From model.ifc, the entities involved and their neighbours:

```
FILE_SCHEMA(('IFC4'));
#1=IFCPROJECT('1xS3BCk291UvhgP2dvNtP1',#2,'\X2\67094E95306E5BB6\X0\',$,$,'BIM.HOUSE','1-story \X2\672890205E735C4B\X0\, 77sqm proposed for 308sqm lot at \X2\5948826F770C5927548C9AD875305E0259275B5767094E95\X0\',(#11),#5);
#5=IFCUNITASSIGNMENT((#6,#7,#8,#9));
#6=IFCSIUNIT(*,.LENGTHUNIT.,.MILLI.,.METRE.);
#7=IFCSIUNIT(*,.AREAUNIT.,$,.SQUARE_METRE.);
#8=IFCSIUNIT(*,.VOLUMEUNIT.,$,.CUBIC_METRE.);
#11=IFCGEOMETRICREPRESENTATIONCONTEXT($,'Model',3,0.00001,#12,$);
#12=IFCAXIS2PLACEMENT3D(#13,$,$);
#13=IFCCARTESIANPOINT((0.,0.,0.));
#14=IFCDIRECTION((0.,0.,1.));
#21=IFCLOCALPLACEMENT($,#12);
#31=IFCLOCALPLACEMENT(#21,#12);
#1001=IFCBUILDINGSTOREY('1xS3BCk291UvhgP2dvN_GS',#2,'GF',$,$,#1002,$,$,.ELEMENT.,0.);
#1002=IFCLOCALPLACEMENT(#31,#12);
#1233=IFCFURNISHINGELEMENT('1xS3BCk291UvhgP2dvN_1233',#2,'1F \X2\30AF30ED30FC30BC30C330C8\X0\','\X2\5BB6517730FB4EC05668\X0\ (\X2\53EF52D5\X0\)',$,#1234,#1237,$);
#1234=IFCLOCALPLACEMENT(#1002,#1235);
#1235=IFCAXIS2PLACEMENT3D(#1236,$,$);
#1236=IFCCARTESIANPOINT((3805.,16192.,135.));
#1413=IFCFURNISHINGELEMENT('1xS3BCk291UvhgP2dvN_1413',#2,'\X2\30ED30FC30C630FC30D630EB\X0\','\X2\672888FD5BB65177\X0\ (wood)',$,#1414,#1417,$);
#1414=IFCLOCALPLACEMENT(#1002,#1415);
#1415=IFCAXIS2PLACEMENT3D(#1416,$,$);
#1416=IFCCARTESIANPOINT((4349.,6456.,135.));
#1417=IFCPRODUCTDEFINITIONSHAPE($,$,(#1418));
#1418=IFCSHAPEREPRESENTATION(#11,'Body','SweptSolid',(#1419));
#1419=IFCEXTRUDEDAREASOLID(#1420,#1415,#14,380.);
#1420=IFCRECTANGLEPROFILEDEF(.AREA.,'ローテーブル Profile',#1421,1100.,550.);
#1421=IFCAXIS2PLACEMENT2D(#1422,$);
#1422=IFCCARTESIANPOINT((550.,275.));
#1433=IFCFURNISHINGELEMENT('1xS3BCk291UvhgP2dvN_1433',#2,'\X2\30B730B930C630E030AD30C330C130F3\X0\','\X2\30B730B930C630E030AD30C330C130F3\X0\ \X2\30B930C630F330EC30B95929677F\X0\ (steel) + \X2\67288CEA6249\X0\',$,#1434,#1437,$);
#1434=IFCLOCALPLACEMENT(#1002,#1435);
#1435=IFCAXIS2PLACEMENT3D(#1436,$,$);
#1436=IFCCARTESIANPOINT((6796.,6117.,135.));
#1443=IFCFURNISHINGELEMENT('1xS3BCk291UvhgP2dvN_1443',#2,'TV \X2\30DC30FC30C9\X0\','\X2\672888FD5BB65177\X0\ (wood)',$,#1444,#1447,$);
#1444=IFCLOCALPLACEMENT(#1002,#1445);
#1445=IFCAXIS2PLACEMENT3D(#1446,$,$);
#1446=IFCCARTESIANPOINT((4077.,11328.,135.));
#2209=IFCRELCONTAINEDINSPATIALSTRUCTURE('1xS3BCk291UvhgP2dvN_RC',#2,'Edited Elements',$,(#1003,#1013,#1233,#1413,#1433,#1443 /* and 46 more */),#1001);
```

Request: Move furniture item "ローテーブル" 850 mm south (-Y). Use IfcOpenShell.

```python
import ifcopenshell
import ifcopenshell.api.geometry
import ifcopenshell.util.placement
import ifcopenshell.util.unit

model = ifcopenshell.open("model.ifc")
unit_scale = ifcopenshell.util.unit.calculate_unit_scale(model)

item = model.by_guid("1xS3BCk291UvhgP2dvN_1413")
matrix = ifcopenshell.util.placement.get_local_placement(item.ObjectPlacement)
matrix[1, 3] -= 0.85 / unit_scale
ifcopenshell.api.geometry.edit_object_placement(model, product=item, matrix=matrix, is_si=False)

print(ifcopenshell.util.placement.get_local_placement(item.ObjectPlacement).round(3) + 0.0)

model.write("model_updated.ifc")
```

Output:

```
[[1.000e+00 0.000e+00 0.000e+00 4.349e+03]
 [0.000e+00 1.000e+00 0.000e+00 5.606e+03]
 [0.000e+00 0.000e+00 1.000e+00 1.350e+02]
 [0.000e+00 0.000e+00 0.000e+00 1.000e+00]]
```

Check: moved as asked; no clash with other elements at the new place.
